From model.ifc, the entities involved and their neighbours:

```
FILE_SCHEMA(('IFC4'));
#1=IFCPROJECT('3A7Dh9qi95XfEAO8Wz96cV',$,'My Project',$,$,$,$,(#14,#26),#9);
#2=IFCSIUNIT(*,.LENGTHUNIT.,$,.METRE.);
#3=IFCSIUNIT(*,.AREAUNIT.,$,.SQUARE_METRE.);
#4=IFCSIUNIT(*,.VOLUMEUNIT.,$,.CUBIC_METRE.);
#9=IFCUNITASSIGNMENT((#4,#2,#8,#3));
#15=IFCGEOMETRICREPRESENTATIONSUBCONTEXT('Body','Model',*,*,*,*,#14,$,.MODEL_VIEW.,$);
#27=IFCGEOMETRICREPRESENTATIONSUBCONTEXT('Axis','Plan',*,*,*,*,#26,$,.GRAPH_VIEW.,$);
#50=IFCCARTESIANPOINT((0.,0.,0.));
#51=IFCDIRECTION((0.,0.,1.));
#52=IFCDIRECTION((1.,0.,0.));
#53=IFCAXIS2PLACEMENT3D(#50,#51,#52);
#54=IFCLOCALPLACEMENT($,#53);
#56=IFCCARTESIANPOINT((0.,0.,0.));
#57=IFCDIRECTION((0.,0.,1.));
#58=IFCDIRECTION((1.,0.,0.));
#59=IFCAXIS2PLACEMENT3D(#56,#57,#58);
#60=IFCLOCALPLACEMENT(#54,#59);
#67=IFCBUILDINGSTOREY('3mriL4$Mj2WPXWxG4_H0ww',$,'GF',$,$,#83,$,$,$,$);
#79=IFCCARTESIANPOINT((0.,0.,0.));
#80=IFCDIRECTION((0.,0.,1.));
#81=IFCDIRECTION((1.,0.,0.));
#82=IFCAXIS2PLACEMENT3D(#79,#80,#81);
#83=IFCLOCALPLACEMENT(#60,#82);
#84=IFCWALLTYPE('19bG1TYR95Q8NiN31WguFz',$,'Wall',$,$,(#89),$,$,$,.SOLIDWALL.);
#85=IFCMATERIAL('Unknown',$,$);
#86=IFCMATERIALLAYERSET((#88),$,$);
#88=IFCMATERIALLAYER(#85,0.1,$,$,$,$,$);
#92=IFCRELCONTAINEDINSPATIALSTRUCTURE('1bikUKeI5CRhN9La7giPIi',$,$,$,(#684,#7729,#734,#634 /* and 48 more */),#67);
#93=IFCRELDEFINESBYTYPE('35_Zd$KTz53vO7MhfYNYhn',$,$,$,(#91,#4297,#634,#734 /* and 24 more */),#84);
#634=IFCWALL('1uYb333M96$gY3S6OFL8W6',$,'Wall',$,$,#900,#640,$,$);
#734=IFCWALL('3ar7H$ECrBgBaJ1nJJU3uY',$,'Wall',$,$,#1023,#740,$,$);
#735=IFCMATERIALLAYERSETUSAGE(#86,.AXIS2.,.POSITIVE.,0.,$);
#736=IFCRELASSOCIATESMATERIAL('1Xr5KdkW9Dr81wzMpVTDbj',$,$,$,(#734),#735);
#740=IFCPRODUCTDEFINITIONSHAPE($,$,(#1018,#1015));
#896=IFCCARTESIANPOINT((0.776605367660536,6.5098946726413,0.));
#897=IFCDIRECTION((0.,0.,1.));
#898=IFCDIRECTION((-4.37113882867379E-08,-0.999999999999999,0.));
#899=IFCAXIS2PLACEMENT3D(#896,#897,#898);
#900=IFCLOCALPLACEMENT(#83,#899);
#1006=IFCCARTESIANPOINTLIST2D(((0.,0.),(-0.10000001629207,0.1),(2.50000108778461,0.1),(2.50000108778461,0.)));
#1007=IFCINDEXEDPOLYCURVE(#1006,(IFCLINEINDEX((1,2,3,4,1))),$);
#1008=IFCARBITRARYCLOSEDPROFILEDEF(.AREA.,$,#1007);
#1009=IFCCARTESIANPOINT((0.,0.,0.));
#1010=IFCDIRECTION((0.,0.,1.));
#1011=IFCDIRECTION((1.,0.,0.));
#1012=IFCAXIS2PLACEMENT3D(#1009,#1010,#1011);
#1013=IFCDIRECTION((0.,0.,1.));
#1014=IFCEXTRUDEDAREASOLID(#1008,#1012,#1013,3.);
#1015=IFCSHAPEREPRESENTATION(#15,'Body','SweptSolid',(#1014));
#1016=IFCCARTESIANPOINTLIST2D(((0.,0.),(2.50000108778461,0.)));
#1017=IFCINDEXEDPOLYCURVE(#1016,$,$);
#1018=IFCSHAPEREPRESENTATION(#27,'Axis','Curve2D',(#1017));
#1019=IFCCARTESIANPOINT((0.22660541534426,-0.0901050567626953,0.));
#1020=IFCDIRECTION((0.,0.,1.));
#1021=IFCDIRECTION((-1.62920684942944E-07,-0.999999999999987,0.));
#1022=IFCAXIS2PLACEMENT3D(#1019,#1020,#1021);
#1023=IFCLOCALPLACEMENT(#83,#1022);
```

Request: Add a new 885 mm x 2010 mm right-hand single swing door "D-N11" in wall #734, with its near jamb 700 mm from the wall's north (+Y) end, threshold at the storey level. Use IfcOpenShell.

```python
import numpy as np
import ifcopenshell
import ifcopenshell.api.feature
import ifcopenshell.api.geometry
import ifcopenshell.api.root
import ifcopenshell.api.spatial
import ifcopenshell.geom
import ifcopenshell.util.element
import ifcopenshell.util.placement
import ifcopenshell.util.representation
import ifcopenshell.util.shape
import ifcopenshell.util.unit

model = ifcopenshell.open("model.ifc")
unit_scale = ifcopenshell.util.unit.calculate_unit_scale(model)
settings = ifcopenshell.geom.settings()


def volume(element):
    """Net volume in cubic metres, openings subtracted."""
    shape = ifcopenshell.geom.create_shape(settings, element)
    return ifcopenshell.util.shape.get_volume(shape.geometry)


wall = model.by_id(734)
storey = ifcopenshell.util.element.get_container(wall, ifc_class="IfcBuildingStorey")
context = ifcopenshell.util.representation.get_context(model, "Model", "Body", "MODEL_VIEW")
before = volume(wall)

width, height, from_end, sill = 0.885, 2.01, 0.7, 0.0  # metres

# The wall runs along its own X axis, and the end named is its -X end.
wall_shape = ifcopenshell.geom.create_shape(settings, wall)
x, y, z = ifcopenshell.util.shape.get_vertices(wall_shape.geometry).T
start = x.min() + from_end
face, thickness = float(y.min()), float(y.max() - y.min())
wall_matrix = ifcopenshell.util.placement.get_local_placement(wall.ObjectPlacement)
level = ifcopenshell.util.placement.get_local_placement(storey.ObjectPlacement)[2, 3]


def in_wall(x, y):
    """Placement at x, y metres in the wall's axes, at sill height."""
    matrix = wall_matrix.copy()
    matrix[:, 3] = wall_matrix @ np.array([x / unit_scale, y / unit_scale, 0.0, 1.0])
    matrix[2, 3] = level + sill / unit_scale
    return matrix


# Opening: a box that overshoots both wall faces by 50 mm.
opening = ifcopenshell.api.root.create_entity(model, ifc_class="IfcOpeningElement", predefined_type="OPENING")
box = ifcopenshell.api.geometry.add_wall_representation(
    model, context=context, length=width, height=height, thickness=thickness + 0.1
)
ifcopenshell.api.geometry.assign_representation(model, product=opening, representation=box)
ifcopenshell.api.geometry.edit_object_placement(model, product=opening, matrix=in_wall(start, face - 0.05), is_si=False)
ifcopenshell.api.feature.add_feature(model, feature=opening, element=wall)

door = ifcopenshell.api.root.create_entity(model, ifc_class="IfcDoor", name="D-N11", predefined_type="DOOR")
door.OverallWidth, door.OverallHeight = width / unit_scale, height / unit_scale
door.OperationType = "SINGLE_SWING_RIGHT"
body = ifcopenshell.api.geometry.add_door_representation(
    model,
    context=context,
    overall_width=door.OverallWidth,
    overall_height=door.OverallHeight,
    operation_type="SINGLE_SWING_RIGHT",
    lining_properties={"LiningDepth": thickness / unit_scale, "ThresholdDepth": thickness / unit_scale},
)
ifcopenshell.api.geometry.assign_representation(model, product=door, representation=body)
ifcopenshell.api.spatial.assign_container(model, products=[door], relating_structure=storey)
ifcopenshell.api.feature.add_filling(model, opening=opening, element=door)

# The lining spans the wall, so the door starts at the wall face.
ifcopenshell.api.geometry.edit_object_placement(model, product=door, matrix=in_wall(start, face), is_si=False)

after = volume(wall)

print(f"wall volume {before:.3f} -> {after:.3f} m3")

model.write("model_rev.ifc")
```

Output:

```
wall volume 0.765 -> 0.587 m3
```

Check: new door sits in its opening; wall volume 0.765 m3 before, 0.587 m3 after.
